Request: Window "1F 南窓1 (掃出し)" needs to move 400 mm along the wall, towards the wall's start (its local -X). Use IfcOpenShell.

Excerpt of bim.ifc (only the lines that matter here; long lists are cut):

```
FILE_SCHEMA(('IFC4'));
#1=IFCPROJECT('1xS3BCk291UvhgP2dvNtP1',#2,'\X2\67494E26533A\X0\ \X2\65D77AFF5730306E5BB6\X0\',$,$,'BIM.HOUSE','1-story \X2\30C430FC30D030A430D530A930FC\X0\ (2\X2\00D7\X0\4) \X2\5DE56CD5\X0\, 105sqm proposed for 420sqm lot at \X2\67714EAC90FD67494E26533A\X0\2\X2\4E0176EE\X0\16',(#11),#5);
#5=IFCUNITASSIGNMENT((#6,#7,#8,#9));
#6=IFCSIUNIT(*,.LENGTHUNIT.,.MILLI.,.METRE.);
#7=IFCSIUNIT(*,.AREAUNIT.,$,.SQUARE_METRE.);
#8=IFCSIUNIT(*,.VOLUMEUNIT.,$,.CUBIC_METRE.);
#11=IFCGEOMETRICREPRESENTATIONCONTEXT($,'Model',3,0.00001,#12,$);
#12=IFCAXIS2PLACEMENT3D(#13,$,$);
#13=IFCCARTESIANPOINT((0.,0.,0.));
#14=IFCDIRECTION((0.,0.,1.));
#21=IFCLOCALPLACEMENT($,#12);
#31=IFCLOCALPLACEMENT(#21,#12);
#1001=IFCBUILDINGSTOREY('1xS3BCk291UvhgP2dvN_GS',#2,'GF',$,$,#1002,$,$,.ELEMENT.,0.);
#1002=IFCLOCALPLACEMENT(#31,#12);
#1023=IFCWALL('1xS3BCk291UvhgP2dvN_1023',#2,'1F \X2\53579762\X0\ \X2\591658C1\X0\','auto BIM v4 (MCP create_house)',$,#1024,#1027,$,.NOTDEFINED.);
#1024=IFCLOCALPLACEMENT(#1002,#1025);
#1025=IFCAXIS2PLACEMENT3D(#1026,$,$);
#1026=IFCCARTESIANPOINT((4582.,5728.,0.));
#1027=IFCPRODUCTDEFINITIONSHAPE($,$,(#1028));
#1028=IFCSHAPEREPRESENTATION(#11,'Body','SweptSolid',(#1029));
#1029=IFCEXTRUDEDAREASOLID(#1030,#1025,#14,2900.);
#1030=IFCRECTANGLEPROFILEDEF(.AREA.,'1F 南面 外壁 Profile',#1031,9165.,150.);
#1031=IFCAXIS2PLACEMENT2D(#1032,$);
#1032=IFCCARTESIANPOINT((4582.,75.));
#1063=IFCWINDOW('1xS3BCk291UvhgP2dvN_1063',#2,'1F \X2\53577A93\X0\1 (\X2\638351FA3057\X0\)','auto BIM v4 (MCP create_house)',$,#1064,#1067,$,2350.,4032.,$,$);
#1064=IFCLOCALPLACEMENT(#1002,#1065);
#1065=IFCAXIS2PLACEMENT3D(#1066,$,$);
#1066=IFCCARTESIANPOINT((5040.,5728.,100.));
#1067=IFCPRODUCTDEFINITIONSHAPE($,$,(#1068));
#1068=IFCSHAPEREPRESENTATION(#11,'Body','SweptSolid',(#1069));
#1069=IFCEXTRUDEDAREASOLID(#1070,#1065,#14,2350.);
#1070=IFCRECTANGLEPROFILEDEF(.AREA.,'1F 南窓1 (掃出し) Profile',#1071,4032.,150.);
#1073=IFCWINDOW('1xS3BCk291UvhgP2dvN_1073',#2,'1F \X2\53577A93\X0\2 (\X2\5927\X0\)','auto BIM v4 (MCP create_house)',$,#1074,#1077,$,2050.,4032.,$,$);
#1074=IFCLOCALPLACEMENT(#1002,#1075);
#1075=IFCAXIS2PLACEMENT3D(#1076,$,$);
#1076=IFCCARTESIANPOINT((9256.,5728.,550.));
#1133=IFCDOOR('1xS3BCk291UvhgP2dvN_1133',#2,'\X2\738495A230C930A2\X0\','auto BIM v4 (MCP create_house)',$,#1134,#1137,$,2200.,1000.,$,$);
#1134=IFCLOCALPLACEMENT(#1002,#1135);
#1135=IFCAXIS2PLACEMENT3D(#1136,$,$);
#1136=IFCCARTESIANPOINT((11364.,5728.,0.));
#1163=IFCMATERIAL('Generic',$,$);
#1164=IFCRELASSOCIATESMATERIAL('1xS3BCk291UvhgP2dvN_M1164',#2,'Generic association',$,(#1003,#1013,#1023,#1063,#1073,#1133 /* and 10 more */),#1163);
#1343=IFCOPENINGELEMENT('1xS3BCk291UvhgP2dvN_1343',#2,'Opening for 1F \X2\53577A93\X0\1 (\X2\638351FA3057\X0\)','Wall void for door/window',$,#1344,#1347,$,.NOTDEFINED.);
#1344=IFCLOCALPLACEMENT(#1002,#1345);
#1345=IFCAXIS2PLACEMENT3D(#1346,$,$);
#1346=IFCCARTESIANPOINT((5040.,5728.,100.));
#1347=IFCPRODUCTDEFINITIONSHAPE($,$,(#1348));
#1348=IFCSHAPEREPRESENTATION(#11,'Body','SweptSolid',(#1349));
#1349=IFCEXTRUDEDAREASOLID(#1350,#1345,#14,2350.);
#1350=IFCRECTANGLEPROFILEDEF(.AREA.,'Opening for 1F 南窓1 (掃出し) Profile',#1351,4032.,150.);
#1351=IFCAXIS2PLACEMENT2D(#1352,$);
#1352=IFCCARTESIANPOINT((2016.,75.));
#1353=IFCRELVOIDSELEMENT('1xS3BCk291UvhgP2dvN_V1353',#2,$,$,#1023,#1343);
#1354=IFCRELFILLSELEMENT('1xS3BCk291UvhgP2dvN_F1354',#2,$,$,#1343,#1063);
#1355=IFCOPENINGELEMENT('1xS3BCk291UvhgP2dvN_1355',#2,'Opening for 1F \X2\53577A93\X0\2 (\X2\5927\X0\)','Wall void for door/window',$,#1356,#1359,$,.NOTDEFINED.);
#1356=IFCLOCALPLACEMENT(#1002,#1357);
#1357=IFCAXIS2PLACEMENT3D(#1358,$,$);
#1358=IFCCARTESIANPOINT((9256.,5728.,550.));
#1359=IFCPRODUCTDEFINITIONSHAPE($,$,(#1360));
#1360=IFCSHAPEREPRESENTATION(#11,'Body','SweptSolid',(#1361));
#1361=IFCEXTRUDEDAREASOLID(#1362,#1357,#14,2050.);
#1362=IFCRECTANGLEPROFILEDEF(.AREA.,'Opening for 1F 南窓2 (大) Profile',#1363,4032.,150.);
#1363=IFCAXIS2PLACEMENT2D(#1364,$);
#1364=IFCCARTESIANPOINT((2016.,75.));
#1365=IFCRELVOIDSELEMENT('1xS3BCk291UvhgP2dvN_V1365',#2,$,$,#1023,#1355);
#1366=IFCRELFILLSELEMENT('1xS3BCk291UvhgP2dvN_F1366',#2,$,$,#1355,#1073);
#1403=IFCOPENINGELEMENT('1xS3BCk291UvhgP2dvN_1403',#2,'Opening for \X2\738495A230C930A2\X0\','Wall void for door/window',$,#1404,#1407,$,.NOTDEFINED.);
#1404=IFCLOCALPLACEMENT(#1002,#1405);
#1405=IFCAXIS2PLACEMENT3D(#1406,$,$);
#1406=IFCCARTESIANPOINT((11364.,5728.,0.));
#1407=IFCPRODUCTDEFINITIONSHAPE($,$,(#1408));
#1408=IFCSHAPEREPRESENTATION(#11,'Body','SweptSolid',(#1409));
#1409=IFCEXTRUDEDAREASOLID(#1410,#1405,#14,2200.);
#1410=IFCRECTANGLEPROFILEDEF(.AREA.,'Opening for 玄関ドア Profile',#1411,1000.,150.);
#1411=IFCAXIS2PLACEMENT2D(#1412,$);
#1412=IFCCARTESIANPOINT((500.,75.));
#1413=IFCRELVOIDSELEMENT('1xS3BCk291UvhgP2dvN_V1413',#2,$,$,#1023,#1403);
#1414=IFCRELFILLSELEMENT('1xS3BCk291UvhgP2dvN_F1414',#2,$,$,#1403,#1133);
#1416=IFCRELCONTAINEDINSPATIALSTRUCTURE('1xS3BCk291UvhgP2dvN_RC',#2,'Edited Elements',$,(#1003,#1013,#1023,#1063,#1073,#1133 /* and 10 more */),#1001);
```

```python
import ifcopenshell
import ifcopenshell.api.geometry
import ifcopenshell.util.placement

model = ifcopenshell.open("bim.ifc")

window = model.by_id(1063)
opening = window.FillsVoids[0].RelatingOpeningElement
wall = opening.VoidsElements[0].RelatingBuildingElement

wall_matrix = ifcopenshell.util.placement.get_local_placement(wall.ObjectPlacement)
shift = wall_matrix[:3, 0] * -400.0
before = ifcopenshell.util.placement.get_local_placement(window.ObjectPlacement)[:3, 3].copy()

# The window is not placed relative to its opening, so move both.
for product in (opening, window):
    matrix = ifcopenshell.util.placement.get_local_placement(product.ObjectPlacement)
    matrix[:3, 3] += shift
    ifcopenshell.api.geometry.edit_object_placement(model, product=product, matrix=matrix, is_si=False)

after = ifcopenshell.util.placement.get_local_placement(window.ObjectPlacement)[:3, 3]
print("window moved by", (after - before).round(3) + 0.0)

model.write("bim_v2.ifc")
```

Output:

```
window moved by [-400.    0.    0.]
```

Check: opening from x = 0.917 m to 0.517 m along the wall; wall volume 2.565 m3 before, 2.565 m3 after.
